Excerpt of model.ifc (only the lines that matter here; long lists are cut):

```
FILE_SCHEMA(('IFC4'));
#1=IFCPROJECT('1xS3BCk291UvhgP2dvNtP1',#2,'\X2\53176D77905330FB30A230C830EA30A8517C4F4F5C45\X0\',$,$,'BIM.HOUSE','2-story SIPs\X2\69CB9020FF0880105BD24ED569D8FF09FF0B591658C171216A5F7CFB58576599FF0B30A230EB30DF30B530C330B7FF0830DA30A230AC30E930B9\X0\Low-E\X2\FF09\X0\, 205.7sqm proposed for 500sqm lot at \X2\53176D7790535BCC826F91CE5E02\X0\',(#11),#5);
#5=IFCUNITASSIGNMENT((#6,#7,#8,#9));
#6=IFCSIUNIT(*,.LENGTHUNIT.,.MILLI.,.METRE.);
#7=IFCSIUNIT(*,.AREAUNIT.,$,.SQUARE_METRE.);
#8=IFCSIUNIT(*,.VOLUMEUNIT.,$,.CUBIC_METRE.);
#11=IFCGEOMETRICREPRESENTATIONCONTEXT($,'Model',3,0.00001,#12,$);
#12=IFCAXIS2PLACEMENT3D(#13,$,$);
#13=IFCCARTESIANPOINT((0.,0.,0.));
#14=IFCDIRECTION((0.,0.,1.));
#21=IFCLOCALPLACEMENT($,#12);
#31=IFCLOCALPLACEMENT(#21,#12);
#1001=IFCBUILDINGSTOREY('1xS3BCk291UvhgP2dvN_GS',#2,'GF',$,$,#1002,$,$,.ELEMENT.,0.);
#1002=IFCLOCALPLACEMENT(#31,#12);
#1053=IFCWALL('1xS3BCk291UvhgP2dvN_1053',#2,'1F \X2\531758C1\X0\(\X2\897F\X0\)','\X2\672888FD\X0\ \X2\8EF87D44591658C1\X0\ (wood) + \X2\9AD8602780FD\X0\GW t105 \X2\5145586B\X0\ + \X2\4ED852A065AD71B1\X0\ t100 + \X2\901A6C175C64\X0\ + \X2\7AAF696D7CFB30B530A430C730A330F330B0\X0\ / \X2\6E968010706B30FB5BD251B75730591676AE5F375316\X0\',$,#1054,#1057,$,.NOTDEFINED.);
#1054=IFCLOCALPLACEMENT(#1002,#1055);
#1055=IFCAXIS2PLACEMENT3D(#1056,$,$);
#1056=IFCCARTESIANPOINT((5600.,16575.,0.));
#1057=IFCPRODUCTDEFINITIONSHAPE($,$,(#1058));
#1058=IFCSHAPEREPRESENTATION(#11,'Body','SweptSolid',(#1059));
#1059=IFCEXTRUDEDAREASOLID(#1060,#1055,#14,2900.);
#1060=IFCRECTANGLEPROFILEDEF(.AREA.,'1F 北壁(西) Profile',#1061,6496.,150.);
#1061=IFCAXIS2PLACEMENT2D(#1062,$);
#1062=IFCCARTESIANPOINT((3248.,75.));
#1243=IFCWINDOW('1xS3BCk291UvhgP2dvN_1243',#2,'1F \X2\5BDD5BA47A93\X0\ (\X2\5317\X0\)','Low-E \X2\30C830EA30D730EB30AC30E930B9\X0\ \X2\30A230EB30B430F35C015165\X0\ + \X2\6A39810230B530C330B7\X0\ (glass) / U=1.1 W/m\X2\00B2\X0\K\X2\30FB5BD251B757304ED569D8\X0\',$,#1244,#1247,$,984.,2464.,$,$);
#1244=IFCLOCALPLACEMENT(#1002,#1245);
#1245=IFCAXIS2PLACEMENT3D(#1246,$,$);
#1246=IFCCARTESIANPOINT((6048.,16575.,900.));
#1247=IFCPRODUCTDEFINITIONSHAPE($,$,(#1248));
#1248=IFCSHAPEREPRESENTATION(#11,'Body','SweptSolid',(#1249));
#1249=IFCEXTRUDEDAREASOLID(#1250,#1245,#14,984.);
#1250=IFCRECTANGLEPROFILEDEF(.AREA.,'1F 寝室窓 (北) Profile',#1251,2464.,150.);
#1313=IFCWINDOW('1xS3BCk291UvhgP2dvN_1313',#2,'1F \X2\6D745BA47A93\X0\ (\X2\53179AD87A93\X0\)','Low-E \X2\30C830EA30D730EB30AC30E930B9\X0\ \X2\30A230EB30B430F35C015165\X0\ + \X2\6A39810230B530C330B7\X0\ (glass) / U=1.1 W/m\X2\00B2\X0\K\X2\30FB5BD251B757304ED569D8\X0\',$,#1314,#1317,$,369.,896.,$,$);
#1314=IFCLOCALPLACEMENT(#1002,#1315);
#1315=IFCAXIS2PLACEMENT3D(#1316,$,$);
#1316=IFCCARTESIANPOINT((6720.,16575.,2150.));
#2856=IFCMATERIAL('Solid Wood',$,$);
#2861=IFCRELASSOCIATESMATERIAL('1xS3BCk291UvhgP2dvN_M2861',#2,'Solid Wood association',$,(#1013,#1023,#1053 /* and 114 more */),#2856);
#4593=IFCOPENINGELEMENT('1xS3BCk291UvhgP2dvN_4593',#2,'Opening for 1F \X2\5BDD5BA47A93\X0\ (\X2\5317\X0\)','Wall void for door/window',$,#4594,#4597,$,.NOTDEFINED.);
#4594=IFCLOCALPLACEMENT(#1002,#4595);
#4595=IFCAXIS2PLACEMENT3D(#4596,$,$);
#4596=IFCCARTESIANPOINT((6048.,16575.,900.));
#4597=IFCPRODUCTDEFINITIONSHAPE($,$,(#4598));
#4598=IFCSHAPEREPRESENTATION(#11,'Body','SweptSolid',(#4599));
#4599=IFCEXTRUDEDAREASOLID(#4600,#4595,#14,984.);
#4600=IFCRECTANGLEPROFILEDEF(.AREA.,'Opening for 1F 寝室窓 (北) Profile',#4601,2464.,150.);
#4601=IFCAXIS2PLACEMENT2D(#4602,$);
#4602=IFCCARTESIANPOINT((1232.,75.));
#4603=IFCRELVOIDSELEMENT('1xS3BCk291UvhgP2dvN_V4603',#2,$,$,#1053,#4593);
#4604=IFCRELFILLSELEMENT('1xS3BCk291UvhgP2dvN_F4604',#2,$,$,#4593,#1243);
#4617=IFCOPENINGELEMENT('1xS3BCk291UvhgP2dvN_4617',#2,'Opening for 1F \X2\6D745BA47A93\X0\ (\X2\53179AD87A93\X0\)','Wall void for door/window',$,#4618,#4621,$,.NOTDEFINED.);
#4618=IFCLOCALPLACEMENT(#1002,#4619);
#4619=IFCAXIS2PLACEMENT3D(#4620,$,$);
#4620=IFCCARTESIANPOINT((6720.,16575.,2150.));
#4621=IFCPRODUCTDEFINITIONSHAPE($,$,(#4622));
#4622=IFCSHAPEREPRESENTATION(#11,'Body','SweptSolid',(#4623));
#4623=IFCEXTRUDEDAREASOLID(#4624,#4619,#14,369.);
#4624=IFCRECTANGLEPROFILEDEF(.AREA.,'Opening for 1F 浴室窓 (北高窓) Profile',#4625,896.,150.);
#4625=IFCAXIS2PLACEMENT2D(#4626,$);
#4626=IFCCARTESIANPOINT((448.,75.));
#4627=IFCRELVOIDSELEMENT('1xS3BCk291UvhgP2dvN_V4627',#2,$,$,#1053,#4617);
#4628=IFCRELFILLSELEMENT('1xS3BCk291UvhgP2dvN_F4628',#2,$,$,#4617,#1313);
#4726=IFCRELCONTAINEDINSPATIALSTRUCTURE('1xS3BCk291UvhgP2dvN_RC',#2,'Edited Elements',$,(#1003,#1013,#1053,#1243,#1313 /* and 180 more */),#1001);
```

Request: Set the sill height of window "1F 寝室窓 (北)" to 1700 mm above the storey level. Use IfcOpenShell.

```python
import numpy as np
import ifcopenshell
import ifcopenshell.api.geometry
import ifcopenshell.geom
import ifcopenshell.util.element
import ifcopenshell.util.placement
import ifcopenshell.util.shape
import ifcopenshell.util.unit

model = ifcopenshell.open("model.ifc")
unit_scale = ifcopenshell.util.unit.calculate_unit_scale(model)

window = model.by_id(1243)
opening = window.FillsVoids[0].RelatingOpeningElement
storey = ifcopenshell.util.element.get_container(window, ifc_class="IfcBuildingStorey")
level = ifcopenshell.util.placement.get_local_placement(storey.ObjectPlacement)[2, 3]

# The opening's origin need not be at the sill, so measure its lowest point.
shape = ifcopenshell.geom.create_shape(ifcopenshell.geom.settings(), opening)
bottom = ifcopenshell.util.shape.get_shape_bottom_elevation(shape, shape.geometry) / unit_scale
dz = level + 1.7 / unit_scale - bottom

shift = np.array([0.0, 0.0, dz])
# The window is not placed relative to its opening, so move both.
for product in (opening, window):
    matrix = ifcopenshell.util.placement.get_local_placement(product.ObjectPlacement)
    matrix[:3, 3] += shift
    ifcopenshell.api.geometry.edit_object_placement(model, product=product, matrix=matrix, is_si=False)

print(f"moved by {dz * unit_scale:+.3f} m")

model.write("model_edited.ifc")
```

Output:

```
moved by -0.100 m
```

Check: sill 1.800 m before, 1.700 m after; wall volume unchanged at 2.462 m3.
